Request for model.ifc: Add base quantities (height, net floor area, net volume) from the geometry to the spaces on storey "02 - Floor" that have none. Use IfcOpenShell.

First a look at what the model holds.

```python
import ifcopenshell
import ifcopenshell.util.element
import ifcopenshell.util.unit

model = ifcopenshell.open("model.ifc")
print(model.schema)
for unit_type in ("LENGTHUNIT", "AREAUNIT", "VOLUMEUNIT"):
    print(unit_type, ifcopenshell.util.unit.calculate_unit_scale(model, unit_type))
storey = next(s for s in model.by_type("IfcBuildingStorey") if s.Name == "02 - Floor")
spaces = [e for e in ifcopenshell.util.element.get_decomposition(storey) if e.is_a("IfcSpace")]
for e in sorted(spaces, key=lambda e: e.id()):
    print(e.id(), e.is_a(), e.Name, list(ifcopenshell.util.element.get_psets(e, qtos_only=True)), sep=" | ")
```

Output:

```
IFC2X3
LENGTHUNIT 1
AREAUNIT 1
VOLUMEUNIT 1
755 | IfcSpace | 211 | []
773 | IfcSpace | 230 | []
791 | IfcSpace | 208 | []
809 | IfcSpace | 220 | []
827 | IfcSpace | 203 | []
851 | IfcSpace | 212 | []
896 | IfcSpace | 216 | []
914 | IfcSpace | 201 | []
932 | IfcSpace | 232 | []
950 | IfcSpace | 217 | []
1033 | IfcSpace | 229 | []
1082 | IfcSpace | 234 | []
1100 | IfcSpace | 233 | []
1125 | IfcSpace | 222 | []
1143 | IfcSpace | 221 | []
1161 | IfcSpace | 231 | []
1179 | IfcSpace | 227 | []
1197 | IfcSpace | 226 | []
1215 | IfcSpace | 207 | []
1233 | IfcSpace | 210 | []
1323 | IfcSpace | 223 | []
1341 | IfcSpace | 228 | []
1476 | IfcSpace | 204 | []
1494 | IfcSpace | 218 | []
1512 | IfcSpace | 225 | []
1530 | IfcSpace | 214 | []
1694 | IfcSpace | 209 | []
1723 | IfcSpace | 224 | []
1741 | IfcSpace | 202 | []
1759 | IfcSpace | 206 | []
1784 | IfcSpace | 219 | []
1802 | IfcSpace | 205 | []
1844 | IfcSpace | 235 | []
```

```python
import ifcopenshell
import ifcopenshell.api.pset
import ifcopenshell.geom
import ifcopenshell.util.element
import ifcopenshell.util.shape
import ifcopenshell.util.unit

model = ifcopenshell.open("model.ifc")
unit_scale = ifcopenshell.util.unit.calculate_unit_scale(model)
area_scale = ifcopenshell.util.unit.calculate_unit_scale(model, "AREAUNIT")
volume_scale = ifcopenshell.util.unit.calculate_unit_scale(model, "VOLUMEUNIT")
settings = ifcopenshell.geom.settings()

storey = next(s for s in model.by_type("IfcBuildingStorey") if s.Name == "02 - Floor")
spaces = [e for e in ifcopenshell.util.element.get_decomposition(storey) if e.is_a("IfcSpace")]

for e in sorted(spaces, key=lambda e: e.id()):
    if ifcopenshell.util.element.get_psets(e, qtos_only=True, should_inherit=False):
        continue
    # Geometry comes back in metres, in the element's own axes.
    shape = ifcopenshell.geom.create_shape(settings, e)
    values = {
        "Height": ifcopenshell.util.shape.get_z(shape.geometry) / unit_scale,
        "NetFloorArea": ifcopenshell.util.shape.get_footprint_area(shape.geometry) / area_scale,
        "NetVolume": ifcopenshell.util.shape.get_volume(shape.geometry) / volume_scale,
    }
    qto = ifcopenshell.api.pset.add_qto(model, product=e, name="BaseQuantities")
    ifcopenshell.api.pset.edit_qto(model, qto=qto, properties=values)
    print(e.id(), {k: round(v, 3) for k, v in values.items()})

model.write("model-out.ifc")
```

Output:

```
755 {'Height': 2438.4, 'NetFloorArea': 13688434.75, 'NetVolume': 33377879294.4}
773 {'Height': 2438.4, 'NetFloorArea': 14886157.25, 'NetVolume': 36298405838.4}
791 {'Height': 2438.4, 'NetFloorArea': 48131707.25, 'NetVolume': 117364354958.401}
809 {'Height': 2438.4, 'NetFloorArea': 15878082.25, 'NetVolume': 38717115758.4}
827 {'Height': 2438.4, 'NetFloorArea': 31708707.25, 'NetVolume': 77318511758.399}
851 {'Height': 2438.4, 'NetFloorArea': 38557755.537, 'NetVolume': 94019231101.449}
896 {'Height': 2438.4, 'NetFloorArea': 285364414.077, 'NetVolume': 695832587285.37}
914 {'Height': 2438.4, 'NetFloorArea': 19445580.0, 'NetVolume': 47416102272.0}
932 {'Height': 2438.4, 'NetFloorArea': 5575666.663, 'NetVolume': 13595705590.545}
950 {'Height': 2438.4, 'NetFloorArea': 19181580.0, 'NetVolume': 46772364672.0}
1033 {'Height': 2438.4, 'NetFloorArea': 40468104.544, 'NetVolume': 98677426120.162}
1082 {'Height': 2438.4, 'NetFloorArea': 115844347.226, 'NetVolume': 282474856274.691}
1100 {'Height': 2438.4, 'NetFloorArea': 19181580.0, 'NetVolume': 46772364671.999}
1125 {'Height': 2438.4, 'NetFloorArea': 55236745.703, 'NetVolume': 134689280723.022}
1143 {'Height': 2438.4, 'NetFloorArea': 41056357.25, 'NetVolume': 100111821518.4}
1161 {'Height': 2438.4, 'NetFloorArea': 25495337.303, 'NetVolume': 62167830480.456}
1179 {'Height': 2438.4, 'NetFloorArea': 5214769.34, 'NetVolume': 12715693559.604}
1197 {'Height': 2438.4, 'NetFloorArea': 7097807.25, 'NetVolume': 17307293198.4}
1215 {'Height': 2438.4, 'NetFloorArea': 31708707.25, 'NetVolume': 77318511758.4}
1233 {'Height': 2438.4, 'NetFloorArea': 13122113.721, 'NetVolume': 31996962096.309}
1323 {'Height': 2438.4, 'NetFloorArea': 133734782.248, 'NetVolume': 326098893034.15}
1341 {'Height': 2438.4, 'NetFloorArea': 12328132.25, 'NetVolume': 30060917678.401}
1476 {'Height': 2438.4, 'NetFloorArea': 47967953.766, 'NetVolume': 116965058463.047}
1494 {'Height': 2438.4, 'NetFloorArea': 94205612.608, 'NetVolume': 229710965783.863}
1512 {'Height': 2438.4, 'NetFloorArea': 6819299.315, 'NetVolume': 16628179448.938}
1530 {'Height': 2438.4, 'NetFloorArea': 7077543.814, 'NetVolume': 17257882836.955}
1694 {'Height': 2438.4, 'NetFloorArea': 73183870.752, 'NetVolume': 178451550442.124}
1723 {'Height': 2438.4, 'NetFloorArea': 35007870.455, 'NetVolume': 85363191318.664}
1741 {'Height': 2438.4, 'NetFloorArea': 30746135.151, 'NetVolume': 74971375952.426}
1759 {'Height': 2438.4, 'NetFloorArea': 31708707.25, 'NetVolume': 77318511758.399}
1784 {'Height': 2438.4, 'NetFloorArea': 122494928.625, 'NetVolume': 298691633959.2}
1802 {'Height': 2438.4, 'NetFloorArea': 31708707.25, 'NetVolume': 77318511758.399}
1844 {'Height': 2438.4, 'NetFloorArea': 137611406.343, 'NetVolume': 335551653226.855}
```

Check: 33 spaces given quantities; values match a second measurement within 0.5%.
